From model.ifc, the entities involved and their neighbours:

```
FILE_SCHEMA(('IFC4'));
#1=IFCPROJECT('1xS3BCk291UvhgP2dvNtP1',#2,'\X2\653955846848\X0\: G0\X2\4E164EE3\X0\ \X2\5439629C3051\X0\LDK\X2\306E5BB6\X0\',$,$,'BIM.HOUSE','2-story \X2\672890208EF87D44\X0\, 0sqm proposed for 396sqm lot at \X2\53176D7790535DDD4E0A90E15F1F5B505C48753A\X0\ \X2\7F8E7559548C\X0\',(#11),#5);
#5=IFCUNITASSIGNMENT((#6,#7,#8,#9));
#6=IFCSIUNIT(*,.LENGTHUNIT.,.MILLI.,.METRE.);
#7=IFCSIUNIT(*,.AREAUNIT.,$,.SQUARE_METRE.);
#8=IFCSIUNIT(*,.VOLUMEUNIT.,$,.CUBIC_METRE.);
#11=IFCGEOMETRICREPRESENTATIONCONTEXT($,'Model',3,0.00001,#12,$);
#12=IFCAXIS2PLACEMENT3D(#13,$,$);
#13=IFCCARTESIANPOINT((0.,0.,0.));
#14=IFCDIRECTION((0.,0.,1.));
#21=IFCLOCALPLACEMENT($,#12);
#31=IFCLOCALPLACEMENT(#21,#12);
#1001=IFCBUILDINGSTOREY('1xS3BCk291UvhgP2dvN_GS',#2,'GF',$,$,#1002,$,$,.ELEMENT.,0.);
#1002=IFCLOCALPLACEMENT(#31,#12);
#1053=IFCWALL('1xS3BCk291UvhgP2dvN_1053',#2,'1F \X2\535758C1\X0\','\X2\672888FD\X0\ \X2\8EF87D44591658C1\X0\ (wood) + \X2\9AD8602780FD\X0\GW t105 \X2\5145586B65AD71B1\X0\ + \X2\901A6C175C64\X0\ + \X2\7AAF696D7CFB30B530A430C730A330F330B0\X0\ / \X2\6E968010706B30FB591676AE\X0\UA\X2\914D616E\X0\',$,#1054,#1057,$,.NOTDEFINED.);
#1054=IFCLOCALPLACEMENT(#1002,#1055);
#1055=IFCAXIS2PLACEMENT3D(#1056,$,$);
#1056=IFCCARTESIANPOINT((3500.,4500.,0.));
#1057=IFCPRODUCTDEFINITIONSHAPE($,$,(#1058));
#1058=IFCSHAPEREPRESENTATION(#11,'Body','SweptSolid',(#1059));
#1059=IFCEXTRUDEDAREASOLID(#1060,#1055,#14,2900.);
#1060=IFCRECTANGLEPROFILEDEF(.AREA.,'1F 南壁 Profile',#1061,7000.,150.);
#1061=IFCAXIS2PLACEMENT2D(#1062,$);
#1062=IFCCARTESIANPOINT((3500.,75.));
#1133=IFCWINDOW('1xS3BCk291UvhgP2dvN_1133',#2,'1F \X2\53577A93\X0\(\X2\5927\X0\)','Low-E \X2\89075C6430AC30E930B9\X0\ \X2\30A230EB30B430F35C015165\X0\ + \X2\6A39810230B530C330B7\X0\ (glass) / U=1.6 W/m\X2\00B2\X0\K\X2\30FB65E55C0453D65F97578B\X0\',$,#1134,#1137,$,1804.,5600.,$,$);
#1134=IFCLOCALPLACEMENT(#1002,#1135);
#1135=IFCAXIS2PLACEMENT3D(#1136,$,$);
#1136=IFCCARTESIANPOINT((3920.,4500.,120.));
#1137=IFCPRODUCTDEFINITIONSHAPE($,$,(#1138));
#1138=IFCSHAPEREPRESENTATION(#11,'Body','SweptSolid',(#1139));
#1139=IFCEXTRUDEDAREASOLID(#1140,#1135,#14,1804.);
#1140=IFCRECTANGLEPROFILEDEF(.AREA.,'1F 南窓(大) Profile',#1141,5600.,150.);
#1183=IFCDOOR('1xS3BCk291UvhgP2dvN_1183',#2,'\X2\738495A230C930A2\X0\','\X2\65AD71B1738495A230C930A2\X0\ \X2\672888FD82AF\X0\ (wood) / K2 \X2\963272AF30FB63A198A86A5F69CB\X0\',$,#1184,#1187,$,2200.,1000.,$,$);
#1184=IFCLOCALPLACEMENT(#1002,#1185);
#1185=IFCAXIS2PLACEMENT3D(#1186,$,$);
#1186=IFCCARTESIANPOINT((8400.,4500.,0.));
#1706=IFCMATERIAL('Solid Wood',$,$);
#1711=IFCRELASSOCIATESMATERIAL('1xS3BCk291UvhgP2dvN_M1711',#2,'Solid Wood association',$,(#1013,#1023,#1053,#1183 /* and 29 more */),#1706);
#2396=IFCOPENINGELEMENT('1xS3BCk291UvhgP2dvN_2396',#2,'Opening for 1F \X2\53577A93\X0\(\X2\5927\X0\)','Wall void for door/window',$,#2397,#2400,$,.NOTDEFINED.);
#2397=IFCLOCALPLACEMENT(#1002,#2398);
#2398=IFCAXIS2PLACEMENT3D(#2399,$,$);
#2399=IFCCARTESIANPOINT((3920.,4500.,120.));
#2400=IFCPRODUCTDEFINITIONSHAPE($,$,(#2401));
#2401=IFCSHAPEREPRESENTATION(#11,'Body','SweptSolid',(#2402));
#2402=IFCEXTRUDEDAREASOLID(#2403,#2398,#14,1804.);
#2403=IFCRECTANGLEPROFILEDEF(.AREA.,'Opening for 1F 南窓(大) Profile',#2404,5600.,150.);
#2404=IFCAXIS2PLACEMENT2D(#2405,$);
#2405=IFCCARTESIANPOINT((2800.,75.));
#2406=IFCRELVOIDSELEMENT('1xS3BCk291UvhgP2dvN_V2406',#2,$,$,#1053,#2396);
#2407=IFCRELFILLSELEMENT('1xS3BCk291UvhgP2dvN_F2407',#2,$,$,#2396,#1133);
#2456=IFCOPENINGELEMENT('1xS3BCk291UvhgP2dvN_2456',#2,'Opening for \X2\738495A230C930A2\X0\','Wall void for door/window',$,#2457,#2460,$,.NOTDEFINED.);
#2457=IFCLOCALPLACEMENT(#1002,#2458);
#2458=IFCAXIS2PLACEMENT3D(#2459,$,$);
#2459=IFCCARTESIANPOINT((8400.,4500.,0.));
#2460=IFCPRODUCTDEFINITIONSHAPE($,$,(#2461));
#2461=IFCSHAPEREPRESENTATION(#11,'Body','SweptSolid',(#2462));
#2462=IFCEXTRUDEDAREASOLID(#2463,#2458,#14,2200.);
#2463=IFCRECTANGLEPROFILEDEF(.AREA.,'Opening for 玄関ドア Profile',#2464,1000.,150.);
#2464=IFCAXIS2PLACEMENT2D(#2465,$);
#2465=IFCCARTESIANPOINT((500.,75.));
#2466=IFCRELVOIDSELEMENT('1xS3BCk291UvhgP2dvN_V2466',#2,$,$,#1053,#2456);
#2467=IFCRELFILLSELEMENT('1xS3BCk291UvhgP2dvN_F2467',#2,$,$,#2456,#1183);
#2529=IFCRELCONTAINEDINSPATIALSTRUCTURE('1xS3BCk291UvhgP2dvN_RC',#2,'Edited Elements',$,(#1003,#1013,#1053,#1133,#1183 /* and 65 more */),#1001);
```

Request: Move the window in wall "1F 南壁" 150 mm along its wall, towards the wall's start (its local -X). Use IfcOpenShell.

```python
import ifcopenshell
import ifcopenshell.api.geometry
import ifcopenshell.util.placement

model = ifcopenshell.open("model.ifc")

window = model.by_id(1133)
opening = window.FillsVoids[0].RelatingOpeningElement
wall = opening.VoidsElements[0].RelatingBuildingElement

wall_matrix = ifcopenshell.util.placement.get_local_placement(wall.ObjectPlacement)
shift = wall_matrix[:3, 0] * -150.0
before = ifcopenshell.util.placement.get_local_placement(window.ObjectPlacement)[:3, 3].copy()

# The window is not placed relative to its opening, so move both.
for product in (opening, window):
    matrix = ifcopenshell.util.placement.get_local_placement(product.ObjectPlacement)
    matrix[:3, 3] += shift
    ifcopenshell.api.geometry.edit_object_placement(model, product=product, matrix=matrix, is_si=False)

after = ifcopenshell.util.placement.get_local_placement(window.ObjectPlacement)[:3, 3]
print("window moved by", (after - before).round(3) + 0.0)

model.write("model_updated.ifc")
```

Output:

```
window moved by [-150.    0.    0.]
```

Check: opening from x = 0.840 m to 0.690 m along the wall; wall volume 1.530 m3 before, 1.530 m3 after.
